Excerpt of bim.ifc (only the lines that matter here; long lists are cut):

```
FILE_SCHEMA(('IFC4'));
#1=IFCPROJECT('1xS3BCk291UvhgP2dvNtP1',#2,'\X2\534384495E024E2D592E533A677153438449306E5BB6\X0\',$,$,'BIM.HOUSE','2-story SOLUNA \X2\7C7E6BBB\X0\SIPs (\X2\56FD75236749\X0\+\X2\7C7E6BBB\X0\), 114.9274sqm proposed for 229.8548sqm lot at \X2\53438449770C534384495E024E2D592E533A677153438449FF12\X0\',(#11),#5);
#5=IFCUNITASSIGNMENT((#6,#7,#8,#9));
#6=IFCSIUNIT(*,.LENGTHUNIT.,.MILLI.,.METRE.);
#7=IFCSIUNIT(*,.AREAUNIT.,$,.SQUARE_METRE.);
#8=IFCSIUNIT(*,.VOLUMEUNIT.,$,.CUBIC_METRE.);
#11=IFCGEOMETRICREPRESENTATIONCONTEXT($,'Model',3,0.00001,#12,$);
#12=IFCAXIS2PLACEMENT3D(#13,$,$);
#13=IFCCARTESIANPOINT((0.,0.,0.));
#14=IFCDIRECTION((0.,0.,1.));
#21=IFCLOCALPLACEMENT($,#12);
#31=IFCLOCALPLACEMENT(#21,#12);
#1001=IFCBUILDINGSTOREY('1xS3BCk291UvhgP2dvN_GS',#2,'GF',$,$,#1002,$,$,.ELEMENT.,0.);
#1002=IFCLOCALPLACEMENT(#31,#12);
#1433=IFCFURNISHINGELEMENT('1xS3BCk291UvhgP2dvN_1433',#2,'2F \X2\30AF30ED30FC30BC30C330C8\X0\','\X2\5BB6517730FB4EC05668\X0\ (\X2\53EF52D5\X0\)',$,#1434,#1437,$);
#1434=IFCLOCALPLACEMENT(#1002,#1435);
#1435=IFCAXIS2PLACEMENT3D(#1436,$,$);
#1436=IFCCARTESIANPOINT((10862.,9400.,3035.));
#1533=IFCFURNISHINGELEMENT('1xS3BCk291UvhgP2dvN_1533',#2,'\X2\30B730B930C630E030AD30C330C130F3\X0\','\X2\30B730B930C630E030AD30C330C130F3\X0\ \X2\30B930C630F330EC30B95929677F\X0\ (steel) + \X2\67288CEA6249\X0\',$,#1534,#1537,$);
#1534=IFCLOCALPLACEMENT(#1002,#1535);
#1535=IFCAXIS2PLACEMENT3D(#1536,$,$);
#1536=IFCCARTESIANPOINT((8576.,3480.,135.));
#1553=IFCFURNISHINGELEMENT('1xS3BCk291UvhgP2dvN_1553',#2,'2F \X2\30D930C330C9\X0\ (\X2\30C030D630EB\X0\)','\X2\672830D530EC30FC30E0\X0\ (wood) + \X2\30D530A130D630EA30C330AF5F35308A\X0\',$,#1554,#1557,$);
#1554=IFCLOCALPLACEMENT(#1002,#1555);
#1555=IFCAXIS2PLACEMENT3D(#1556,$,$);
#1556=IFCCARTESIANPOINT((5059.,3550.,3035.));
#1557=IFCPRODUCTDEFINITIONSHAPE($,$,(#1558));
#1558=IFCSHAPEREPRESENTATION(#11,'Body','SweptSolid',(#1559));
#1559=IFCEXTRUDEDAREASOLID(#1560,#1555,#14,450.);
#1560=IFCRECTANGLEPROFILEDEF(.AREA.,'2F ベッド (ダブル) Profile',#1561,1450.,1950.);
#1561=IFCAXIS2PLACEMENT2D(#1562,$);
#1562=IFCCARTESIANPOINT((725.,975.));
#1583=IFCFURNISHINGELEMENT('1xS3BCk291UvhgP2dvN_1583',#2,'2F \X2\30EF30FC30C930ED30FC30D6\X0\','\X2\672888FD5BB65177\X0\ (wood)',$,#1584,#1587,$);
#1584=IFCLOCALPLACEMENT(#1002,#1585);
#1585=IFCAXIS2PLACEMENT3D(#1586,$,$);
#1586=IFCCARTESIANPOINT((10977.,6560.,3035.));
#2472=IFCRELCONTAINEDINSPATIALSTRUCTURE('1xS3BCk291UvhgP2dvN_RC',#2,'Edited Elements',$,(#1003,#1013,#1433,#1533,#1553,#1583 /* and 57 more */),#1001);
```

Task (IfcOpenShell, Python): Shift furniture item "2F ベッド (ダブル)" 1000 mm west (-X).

```python
import ifcopenshell
import ifcopenshell.api.geometry
import ifcopenshell.util.placement

model = ifcopenshell.open("bim.ifc")

item = model.by_id(1553)
matrix = ifcopenshell.util.placement.get_local_placement(item.ObjectPlacement)
matrix[0, 3] -= 1000.0
ifcopenshell.api.geometry.edit_object_placement(model, product=item, matrix=matrix, is_si=False)

print(ifcopenshell.util.placement.get_local_placement(item.ObjectPlacement).round(3) + 0.0)

model.write("bim_v2.ifc")
```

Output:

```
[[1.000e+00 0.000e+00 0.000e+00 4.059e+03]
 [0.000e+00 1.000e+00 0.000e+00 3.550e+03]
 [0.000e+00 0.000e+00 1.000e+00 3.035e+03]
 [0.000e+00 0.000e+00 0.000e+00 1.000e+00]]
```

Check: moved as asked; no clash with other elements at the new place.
